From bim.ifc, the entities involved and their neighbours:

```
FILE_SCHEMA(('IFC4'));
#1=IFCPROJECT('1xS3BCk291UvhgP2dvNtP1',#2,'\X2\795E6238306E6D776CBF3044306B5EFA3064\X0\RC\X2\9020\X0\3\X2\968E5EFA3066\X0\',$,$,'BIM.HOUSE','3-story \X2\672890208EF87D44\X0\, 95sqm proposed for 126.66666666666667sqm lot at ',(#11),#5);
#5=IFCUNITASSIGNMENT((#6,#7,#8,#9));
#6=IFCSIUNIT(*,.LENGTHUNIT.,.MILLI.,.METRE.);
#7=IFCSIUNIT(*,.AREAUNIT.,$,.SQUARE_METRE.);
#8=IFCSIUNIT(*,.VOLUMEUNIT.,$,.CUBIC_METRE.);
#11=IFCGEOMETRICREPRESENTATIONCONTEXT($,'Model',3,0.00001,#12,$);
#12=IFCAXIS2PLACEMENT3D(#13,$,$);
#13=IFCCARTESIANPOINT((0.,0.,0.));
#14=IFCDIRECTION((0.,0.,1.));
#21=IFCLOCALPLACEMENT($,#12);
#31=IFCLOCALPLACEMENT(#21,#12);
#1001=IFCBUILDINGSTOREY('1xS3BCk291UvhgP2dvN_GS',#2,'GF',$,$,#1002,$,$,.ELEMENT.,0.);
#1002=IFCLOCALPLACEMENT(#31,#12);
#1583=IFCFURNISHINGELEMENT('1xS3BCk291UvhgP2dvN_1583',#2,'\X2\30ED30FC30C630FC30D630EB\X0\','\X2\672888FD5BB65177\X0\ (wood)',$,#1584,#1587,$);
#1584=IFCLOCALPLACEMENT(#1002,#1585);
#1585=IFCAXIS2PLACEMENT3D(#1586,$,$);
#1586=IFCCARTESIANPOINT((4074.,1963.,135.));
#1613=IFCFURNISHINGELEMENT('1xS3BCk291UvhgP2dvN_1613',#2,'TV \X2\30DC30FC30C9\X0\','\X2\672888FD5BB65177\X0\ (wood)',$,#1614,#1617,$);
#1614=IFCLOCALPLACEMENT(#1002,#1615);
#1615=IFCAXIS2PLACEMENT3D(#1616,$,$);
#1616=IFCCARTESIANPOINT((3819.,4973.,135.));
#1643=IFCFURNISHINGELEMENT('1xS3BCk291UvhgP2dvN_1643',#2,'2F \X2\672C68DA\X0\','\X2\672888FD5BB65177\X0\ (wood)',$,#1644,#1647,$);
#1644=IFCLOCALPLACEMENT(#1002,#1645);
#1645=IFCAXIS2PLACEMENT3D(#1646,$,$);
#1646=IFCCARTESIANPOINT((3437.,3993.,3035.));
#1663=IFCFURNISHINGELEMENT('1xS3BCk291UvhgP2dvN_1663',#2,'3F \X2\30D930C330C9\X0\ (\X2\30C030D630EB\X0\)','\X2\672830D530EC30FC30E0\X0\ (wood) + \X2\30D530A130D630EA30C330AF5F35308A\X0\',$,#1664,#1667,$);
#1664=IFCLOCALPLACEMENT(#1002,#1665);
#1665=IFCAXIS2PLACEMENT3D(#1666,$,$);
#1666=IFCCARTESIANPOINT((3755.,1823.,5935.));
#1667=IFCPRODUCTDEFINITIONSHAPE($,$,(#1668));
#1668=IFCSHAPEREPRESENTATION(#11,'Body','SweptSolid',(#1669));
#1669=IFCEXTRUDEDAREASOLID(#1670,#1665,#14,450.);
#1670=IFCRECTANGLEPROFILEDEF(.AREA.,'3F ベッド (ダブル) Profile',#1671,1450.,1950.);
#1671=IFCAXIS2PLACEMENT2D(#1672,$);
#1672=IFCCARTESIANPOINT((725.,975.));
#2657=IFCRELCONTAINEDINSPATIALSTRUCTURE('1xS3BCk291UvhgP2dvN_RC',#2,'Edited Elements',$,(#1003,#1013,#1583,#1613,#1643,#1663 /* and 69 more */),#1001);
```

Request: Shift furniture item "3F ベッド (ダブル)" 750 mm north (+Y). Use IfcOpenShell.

```python
import ifcopenshell
import ifcopenshell.api.geometry
import ifcopenshell.util.placement

model = ifcopenshell.open("bim.ifc")

item = model.by_guid("1xS3BCk291UvhgP2dvN_1663")
matrix = ifcopenshell.util.placement.get_local_placement(item.ObjectPlacement)
matrix[1, 3] += 750.0
ifcopenshell.api.geometry.edit_object_placement(model, product=item, matrix=matrix, is_si=False)

print(ifcopenshell.util.placement.get_local_placement(item.ObjectPlacement).round(3) + 0.0)

model.write("bim_edited.ifc")
```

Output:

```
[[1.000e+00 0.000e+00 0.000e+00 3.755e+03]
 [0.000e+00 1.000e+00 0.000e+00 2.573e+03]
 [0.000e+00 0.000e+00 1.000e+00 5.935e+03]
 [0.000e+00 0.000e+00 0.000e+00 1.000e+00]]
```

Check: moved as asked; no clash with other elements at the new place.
